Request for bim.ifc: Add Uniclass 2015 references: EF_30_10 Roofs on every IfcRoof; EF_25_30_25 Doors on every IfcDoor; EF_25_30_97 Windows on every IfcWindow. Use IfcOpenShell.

First a look at what the model holds.

```python
import ifcopenshell

model = ifcopenshell.open("bim.ifc")
print(model.schema)
print("classifications:", [c.Name for c in model.by_type("IfcClassification")])
for ifc_class in ("IfcDoor", "IfcRoof", "IfcStair", "IfcWall", "IfcWindow"):
    print(ifc_class, len(model.by_type(ifc_class)))
```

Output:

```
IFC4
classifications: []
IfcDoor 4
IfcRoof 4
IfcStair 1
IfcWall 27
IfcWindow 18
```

```python
import ifcopenshell
import ifcopenshell.api.classification

model = ifcopenshell.open("bim.ifc")

system = ifcopenshell.api.classification.add_classification(model, classification="Uniclass 2015")

codes = {
    "IfcRoof": ("EF_30_10", "Roofs"),
    "IfcDoor": ("EF_25_30_25", "Doors"),
    "IfcWindow": ("EF_25_30_97", "Windows"),
}
for ifc_class, (code, name) in codes.items():
    products = model.by_type(ifc_class)
    ifcopenshell.api.classification.add_reference(
        model, products=products, classification=system, identification=code, name=name
    )
    print(code, len(products))

model.write("bim-out.ifc")
```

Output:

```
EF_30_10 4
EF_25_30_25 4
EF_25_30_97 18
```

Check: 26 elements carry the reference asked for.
